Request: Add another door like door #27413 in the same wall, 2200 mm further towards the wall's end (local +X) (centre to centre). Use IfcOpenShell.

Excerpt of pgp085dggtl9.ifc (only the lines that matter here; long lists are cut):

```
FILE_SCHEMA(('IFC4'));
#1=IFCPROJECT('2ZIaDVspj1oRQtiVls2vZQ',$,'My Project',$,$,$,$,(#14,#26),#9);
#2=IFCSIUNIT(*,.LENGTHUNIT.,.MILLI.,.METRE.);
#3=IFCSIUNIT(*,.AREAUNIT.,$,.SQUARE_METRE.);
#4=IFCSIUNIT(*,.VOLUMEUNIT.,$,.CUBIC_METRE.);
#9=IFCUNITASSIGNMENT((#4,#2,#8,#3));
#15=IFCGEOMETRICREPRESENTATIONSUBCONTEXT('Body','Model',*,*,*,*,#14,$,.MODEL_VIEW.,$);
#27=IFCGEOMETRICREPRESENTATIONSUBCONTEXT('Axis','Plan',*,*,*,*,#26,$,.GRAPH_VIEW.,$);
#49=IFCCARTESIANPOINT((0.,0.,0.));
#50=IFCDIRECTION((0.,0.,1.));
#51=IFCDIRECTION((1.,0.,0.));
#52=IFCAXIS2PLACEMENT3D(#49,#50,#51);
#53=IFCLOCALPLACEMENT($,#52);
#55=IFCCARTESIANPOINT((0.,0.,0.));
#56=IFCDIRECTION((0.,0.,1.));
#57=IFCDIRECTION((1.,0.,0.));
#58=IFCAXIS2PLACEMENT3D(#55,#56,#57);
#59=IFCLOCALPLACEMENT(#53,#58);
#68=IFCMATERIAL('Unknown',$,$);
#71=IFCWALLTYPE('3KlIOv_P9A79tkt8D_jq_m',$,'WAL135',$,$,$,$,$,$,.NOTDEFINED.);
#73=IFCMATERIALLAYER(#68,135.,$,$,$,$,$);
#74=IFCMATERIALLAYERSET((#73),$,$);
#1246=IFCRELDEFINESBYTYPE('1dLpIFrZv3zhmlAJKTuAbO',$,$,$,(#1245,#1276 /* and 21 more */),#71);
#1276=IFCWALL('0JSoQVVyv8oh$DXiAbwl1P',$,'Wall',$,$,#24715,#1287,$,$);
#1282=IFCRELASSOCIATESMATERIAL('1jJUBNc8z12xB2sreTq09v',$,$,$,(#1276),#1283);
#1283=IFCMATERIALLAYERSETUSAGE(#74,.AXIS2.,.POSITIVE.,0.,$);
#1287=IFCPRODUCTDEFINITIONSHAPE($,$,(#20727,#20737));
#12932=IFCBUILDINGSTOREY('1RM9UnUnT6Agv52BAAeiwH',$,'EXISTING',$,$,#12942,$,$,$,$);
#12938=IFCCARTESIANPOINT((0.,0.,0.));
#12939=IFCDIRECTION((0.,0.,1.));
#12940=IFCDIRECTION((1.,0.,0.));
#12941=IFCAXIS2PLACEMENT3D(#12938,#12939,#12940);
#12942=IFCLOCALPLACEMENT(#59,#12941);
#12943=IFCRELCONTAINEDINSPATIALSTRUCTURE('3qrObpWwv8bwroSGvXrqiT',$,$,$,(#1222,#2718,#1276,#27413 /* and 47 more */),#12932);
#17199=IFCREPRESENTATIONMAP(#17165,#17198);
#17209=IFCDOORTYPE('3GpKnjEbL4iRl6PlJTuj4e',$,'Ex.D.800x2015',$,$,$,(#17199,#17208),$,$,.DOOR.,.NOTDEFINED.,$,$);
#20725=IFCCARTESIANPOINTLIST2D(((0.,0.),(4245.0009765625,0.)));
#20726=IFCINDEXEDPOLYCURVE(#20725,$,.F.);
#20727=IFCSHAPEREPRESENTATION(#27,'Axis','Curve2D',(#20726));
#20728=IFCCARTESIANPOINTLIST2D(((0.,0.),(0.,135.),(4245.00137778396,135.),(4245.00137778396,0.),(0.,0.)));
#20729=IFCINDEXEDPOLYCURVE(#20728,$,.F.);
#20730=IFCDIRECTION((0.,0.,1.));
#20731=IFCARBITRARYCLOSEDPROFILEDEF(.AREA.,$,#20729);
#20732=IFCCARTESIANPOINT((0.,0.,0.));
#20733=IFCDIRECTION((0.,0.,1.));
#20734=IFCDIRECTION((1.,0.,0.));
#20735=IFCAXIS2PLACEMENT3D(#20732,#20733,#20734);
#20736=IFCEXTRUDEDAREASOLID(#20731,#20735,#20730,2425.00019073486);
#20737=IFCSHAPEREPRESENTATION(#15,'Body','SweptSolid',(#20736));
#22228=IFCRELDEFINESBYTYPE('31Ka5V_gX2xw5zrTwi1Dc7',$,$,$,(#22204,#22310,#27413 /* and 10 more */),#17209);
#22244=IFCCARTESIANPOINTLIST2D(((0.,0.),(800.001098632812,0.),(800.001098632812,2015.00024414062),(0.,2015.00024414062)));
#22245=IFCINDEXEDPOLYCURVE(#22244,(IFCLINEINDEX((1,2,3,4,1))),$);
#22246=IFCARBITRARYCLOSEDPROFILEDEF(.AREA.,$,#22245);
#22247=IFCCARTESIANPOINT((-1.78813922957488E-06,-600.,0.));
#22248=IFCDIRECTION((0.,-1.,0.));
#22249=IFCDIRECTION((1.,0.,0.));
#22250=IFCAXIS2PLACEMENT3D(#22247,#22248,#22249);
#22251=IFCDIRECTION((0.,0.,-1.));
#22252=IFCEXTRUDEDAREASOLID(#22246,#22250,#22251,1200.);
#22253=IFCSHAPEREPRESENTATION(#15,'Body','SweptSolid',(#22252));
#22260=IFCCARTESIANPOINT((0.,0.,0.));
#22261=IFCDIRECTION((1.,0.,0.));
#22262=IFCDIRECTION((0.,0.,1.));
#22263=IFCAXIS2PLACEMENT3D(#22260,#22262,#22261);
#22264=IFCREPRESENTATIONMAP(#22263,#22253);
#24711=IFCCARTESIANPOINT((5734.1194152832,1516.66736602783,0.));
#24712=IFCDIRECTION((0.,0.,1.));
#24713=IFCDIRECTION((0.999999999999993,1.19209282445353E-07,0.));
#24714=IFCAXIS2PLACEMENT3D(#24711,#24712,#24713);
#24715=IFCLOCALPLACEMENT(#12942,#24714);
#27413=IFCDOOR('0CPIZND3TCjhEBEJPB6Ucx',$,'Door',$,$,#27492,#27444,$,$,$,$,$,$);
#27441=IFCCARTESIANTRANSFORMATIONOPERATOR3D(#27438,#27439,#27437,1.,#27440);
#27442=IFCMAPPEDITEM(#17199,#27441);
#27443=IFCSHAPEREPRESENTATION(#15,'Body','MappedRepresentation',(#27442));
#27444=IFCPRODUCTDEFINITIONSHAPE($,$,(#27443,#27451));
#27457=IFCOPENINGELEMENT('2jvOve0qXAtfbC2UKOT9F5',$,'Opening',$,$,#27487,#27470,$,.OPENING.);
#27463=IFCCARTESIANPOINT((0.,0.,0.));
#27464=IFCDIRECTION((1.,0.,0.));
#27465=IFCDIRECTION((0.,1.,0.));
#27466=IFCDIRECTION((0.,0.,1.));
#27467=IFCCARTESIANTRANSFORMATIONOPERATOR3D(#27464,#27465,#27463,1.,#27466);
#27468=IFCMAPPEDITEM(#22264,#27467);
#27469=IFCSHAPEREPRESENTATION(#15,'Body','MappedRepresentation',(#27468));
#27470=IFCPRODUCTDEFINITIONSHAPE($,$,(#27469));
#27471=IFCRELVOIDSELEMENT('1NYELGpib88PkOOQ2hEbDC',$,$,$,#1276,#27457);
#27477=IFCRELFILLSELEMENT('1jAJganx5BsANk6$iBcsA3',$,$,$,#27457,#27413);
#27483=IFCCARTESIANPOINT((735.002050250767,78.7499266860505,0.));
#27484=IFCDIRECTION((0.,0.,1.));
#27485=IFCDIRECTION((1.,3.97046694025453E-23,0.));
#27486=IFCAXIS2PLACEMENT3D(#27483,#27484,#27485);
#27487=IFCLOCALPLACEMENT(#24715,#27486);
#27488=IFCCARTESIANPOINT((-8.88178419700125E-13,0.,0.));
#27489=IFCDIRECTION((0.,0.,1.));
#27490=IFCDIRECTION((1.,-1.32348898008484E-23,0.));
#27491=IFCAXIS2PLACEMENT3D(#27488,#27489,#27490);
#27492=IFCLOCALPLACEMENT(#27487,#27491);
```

```python
import ifcopenshell
import ifcopenshell.api.feature
import ifcopenshell.api.geometry
import ifcopenshell.api.root
import ifcopenshell.geom
import ifcopenshell.util.element
import ifcopenshell.util.placement
import ifcopenshell.util.shape
import ifcopenshell.util.unit

model = ifcopenshell.open("pgp085dggtl9.ifc")
unit_scale = ifcopenshell.util.unit.calculate_unit_scale(model)
settings = ifcopenshell.geom.settings()


def volume(element):
    """Net volume in cubic metres, openings subtracted."""
    shape = ifcopenshell.geom.create_shape(settings, element)
    return ifcopenshell.util.shape.get_volume(shape.geometry)


door = model.by_id(27413)
opening = door.FillsVoids[0].RelatingOpeningElement
wall = opening.VoidsElements[0].RelatingBuildingElement
before = volume(wall)
shift = ifcopenshell.util.placement.get_local_placement(wall.ObjectPlacement)[:3, 0] * 2.2 / unit_scale

# copy_class copies the void relationship, type, container and properties, but no geometry.
new_opening = ifcopenshell.api.root.copy_class(model, product=opening)
new_opening.Representation = ifcopenshell.util.element.copy_deep(
    model, opening.Representation, exclude=["IfcGeometricRepresentationContext", "IfcRepresentationMap"]
)
new_door = ifcopenshell.api.root.copy_class(model, product=door)
new_door.Representation = ifcopenshell.util.element.copy_deep(
    model, door.Representation, exclude=["IfcGeometricRepresentationContext", "IfcRepresentationMap"]
)
ifcopenshell.api.feature.add_filling(model, opening=new_opening, element=new_door)

for old, new in ((opening, new_opening), (door, new_door)):
    matrix = ifcopenshell.util.placement.get_local_placement(old.ObjectPlacement)
    matrix[:3, 3] += shift
    ifcopenshell.api.geometry.edit_object_placement(model, product=new, matrix=matrix, is_si=False)

after = volume(wall)

print(f"wall volume {before:.3f} -> {after:.3f} m3")

model.write("pgp085dggtl9_rev.ifc")
```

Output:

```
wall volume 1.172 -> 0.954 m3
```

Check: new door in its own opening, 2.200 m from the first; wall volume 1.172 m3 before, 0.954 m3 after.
